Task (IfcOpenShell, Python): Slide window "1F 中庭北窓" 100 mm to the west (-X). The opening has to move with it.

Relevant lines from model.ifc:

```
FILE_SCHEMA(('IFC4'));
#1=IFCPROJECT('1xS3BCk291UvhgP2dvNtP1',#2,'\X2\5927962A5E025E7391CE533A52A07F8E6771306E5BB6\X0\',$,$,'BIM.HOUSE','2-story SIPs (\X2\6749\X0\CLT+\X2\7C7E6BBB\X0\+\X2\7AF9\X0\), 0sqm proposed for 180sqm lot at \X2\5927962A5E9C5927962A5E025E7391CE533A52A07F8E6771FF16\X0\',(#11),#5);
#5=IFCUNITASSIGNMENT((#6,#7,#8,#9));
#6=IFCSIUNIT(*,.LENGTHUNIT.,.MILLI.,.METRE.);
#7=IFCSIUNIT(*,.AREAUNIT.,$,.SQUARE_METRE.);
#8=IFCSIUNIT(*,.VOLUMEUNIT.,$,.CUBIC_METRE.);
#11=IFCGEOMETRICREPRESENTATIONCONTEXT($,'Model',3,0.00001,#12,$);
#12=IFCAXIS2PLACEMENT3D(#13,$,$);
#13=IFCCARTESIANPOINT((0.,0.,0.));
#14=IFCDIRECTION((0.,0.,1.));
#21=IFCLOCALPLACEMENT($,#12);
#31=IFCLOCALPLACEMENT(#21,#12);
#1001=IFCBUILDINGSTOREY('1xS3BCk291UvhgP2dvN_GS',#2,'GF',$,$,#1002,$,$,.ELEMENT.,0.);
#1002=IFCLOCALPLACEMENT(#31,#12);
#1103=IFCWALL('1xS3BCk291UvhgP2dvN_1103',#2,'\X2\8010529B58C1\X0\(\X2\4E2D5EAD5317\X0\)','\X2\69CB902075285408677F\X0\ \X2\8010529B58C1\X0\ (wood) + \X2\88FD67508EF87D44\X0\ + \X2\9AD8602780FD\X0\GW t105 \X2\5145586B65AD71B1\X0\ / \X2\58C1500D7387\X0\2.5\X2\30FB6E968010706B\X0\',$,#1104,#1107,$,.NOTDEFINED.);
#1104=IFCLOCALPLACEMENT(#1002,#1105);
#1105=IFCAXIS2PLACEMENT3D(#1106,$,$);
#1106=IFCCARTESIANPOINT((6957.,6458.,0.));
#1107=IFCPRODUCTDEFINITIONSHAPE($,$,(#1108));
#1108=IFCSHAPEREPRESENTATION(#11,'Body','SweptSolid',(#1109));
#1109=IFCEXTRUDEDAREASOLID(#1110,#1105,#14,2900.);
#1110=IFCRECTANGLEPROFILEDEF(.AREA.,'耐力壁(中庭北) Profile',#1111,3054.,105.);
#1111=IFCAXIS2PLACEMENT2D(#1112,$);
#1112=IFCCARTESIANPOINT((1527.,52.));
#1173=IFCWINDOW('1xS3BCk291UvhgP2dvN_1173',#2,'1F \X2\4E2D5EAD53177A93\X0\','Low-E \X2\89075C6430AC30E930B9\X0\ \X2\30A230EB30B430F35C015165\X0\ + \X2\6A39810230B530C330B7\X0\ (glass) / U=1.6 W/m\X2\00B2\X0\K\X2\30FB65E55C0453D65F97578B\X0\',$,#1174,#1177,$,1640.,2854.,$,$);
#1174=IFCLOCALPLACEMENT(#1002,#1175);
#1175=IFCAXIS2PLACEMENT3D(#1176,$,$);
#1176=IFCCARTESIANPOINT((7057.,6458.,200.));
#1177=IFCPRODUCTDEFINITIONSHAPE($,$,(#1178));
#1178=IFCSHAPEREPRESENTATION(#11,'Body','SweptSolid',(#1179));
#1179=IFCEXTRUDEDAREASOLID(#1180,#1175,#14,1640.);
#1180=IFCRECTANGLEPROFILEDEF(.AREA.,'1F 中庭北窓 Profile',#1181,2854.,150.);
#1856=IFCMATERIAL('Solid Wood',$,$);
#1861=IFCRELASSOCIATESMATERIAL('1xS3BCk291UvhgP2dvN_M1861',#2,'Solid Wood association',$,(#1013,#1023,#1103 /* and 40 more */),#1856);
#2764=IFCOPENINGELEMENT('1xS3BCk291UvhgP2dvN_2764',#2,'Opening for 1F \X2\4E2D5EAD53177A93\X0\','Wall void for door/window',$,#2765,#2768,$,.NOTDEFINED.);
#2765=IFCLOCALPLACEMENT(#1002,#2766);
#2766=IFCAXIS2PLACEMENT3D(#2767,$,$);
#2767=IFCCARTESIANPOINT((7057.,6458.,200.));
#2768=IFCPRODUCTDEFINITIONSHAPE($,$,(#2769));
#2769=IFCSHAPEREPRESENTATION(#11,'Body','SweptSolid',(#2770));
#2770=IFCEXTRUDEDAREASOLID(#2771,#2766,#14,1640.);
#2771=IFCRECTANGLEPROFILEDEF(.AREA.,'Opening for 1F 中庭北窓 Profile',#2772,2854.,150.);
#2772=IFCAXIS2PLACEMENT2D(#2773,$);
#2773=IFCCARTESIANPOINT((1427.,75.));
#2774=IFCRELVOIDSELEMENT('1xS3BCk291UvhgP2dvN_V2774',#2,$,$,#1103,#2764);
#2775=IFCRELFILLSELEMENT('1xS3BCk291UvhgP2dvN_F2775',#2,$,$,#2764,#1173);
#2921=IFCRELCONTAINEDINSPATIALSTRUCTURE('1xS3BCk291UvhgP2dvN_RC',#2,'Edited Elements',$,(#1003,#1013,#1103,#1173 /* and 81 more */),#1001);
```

```python
import ifcopenshell
import ifcopenshell.api.geometry
import ifcopenshell.util.placement

model = ifcopenshell.open("model.ifc")

window = model.by_guid("1xS3BCk291UvhgP2dvN_1173")
opening = window.FillsVoids[0].RelatingOpeningElement
wall = opening.VoidsElements[0].RelatingBuildingElement

wall_matrix = ifcopenshell.util.placement.get_local_placement(wall.ObjectPlacement)
shift = wall_matrix[:3, 0] * -100.0
before = ifcopenshell.util.placement.get_local_placement(window.ObjectPlacement)[:3, 3].copy()

# The window is not placed relative to its opening, so move both.
for product in (opening, window):
    matrix = ifcopenshell.util.placement.get_local_placement(product.ObjectPlacement)
    matrix[:3, 3] += shift
    ifcopenshell.api.geometry.edit_object_placement(model, product=product, matrix=matrix, is_si=False)

after = ifcopenshell.util.placement.get_local_placement(window.ObjectPlacement)[:3, 3]
print("window moved by", (after - before).round(3) + 0.0)

model.write("model_updated.ifc")
```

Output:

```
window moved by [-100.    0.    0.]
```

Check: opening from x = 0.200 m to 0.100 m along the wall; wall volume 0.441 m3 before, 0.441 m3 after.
